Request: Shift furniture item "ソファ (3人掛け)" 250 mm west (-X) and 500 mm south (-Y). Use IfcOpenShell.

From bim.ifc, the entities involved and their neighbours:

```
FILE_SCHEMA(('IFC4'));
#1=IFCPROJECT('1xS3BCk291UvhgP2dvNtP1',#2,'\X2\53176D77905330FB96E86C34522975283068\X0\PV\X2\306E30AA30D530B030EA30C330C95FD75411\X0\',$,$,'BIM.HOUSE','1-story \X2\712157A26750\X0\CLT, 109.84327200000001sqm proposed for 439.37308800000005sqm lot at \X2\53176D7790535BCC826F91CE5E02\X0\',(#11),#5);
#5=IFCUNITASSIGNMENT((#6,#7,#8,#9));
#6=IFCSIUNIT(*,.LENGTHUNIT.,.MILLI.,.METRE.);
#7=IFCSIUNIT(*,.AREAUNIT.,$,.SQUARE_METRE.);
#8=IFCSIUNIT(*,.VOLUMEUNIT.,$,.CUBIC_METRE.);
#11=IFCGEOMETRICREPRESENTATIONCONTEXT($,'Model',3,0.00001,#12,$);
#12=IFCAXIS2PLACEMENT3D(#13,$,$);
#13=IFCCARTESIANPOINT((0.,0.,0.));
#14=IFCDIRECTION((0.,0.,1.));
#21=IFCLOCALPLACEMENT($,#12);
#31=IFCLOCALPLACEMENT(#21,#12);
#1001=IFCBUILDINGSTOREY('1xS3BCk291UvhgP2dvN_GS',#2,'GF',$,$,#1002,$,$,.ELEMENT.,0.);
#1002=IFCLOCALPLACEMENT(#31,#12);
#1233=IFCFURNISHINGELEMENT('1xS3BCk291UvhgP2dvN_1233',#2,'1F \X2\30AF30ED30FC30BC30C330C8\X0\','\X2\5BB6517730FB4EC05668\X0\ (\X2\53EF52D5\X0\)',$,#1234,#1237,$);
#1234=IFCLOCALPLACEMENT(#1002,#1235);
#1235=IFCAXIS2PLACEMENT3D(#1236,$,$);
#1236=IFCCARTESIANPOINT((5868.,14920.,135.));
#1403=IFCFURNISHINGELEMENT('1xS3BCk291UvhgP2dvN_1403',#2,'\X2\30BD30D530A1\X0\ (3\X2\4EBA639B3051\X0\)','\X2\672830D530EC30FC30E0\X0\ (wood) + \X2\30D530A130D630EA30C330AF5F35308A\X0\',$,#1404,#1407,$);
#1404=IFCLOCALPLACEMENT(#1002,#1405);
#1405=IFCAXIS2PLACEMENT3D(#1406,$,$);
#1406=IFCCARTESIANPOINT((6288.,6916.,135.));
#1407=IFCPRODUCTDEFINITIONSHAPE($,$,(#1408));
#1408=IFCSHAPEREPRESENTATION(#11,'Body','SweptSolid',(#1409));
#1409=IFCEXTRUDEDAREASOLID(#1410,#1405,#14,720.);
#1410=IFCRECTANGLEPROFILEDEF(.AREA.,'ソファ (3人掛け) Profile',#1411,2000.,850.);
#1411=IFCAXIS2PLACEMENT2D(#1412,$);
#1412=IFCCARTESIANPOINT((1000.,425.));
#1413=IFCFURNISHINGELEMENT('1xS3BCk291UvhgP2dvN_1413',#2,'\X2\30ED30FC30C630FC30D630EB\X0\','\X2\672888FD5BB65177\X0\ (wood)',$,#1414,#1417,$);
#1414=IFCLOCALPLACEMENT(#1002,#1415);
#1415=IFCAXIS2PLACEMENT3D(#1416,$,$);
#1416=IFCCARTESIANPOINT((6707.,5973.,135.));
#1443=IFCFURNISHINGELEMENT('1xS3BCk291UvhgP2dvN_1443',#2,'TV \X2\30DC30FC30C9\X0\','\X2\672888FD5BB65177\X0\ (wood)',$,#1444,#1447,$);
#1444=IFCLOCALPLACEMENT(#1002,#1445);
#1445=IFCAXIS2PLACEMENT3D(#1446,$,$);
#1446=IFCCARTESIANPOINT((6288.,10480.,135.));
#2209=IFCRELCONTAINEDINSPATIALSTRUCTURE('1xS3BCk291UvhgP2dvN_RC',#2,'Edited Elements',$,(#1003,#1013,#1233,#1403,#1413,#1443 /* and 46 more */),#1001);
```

```python
import ifcopenshell
import ifcopenshell.api.geometry
import ifcopenshell.util.placement

model = ifcopenshell.open("bim.ifc")

item = model.by_id(1403)
matrix = ifcopenshell.util.placement.get_local_placement(item.ObjectPlacement)
matrix[0, 3] -= 250.0
matrix[1, 3] -= 500.0
ifcopenshell.api.geometry.edit_object_placement(model, product=item, matrix=matrix, is_si=False)

print(ifcopenshell.util.placement.get_local_placement(item.ObjectPlacement).round(3) + 0.0)

model.write("bim_edited.ifc")
```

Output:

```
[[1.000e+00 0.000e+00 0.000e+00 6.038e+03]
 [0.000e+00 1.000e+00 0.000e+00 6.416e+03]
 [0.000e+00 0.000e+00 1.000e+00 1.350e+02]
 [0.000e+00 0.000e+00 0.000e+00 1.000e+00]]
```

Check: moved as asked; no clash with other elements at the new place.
